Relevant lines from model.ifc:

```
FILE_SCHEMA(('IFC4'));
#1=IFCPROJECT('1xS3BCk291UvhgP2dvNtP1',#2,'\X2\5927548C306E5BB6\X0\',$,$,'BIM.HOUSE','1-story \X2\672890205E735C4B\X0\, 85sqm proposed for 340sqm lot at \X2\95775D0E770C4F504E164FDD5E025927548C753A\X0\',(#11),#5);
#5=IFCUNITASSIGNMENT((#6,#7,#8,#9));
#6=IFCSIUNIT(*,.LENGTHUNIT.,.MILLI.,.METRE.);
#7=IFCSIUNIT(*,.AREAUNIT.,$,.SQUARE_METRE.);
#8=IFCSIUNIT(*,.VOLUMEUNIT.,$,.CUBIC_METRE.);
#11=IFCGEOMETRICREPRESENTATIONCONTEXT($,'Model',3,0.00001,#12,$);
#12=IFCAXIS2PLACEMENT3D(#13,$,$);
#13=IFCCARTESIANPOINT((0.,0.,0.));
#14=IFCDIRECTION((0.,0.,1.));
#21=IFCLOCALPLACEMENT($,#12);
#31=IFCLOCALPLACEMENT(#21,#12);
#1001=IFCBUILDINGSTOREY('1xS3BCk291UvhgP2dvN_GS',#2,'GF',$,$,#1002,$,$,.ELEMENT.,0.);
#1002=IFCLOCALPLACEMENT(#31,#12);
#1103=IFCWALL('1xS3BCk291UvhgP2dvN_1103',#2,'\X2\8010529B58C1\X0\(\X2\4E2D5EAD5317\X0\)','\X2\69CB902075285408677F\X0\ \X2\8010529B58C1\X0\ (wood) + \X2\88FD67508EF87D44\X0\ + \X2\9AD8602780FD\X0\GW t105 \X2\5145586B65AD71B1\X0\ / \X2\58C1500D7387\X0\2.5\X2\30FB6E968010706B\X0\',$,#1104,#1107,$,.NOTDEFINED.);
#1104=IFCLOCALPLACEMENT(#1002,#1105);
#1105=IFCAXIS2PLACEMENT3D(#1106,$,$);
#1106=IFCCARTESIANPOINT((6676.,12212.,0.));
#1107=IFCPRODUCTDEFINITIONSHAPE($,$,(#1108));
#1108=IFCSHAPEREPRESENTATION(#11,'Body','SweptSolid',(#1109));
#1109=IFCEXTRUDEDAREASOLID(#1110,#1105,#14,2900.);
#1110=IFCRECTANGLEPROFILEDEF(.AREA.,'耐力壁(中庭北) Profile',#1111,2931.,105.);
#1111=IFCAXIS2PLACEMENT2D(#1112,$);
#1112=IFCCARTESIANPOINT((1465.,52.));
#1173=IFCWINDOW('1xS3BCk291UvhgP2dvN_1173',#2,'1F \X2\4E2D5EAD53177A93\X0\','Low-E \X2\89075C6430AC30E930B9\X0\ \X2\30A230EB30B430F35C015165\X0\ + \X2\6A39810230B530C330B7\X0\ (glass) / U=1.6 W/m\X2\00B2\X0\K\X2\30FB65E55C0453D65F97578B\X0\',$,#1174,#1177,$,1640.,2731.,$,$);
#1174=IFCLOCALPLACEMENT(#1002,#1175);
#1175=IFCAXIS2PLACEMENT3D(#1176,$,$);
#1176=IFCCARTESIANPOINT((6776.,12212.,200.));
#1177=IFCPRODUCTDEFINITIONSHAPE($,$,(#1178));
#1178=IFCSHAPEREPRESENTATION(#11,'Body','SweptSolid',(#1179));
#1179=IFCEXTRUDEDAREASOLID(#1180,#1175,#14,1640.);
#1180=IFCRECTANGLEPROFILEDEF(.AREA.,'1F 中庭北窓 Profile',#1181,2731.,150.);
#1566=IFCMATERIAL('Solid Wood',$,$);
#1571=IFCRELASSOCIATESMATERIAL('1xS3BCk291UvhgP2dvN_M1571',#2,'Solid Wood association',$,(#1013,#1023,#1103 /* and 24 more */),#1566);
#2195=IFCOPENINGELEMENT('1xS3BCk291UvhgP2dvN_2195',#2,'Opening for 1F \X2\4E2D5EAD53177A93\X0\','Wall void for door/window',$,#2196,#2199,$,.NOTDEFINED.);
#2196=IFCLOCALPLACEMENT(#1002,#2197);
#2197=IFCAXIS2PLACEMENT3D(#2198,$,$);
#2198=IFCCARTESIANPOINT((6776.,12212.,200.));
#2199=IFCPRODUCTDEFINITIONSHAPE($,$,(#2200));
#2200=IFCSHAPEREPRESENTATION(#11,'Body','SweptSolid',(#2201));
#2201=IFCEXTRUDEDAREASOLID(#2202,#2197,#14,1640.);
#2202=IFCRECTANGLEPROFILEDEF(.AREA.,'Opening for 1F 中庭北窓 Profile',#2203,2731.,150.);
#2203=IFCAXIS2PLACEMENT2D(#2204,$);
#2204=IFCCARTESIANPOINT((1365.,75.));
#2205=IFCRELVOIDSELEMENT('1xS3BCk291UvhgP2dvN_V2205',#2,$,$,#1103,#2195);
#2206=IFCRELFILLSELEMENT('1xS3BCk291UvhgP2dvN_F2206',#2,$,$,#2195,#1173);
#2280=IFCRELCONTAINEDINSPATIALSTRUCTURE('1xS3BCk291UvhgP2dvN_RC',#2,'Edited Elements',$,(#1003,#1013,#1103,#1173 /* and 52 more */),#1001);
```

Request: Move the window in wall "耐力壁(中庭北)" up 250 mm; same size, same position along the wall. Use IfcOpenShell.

```python
import numpy as np
import ifcopenshell
import ifcopenshell.api.geometry
import ifcopenshell.util.placement
import ifcopenshell.util.unit

model = ifcopenshell.open("model.ifc")
unit_scale = ifcopenshell.util.unit.calculate_unit_scale(model)

window = model.by_guid("1xS3BCk291UvhgP2dvN_1173")
opening = window.FillsVoids[0].RelatingOpeningElement
dz = 0.25 / unit_scale

shift = np.array([0.0, 0.0, dz])
# The window is not placed relative to its opening, so move both.
for product in (opening, window):
    matrix = ifcopenshell.util.placement.get_local_placement(product.ObjectPlacement)
    matrix[:3, 3] += shift
    ifcopenshell.api.geometry.edit_object_placement(model, product=product, matrix=matrix, is_si=False)

print(f"moved by {dz * unit_scale:+.3f} m")

model.write("model_edited.ifc")
```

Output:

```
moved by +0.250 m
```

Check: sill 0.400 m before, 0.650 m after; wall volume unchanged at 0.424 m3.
